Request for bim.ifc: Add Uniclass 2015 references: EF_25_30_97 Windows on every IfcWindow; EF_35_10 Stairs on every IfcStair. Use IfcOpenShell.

First a look at what the model holds.

```python
import ifcopenshell

model = ifcopenshell.open("bim.ifc")
print(model.schema)
print("classifications:", [c.Name for c in model.by_type("IfcClassification")])
for ifc_class in ("IfcDoor", "IfcRoof", "IfcStair", "IfcWall", "IfcWindow"):
    print(ifc_class, len(model.by_type(ifc_class)))
```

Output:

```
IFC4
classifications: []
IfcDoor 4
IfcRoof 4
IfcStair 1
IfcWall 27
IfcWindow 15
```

```python
import ifcopenshell
import ifcopenshell.api.classification

model = ifcopenshell.open("bim.ifc")

system = ifcopenshell.api.classification.add_classification(model, classification="Uniclass 2015")

codes = {
    "IfcWindow": ("EF_25_30_97", "Windows"),
    "IfcStair": ("EF_35_10", "Stairs"),
}
for ifc_class, (code, name) in codes.items():
    products = model.by_type(ifc_class)
    ifcopenshell.api.classification.add_reference(
        model, products=products, classification=system, identification=code, name=name
    )
    print(code, len(products))

model.write("bim_updated.ifc")
```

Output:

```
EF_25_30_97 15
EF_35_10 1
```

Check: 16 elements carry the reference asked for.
